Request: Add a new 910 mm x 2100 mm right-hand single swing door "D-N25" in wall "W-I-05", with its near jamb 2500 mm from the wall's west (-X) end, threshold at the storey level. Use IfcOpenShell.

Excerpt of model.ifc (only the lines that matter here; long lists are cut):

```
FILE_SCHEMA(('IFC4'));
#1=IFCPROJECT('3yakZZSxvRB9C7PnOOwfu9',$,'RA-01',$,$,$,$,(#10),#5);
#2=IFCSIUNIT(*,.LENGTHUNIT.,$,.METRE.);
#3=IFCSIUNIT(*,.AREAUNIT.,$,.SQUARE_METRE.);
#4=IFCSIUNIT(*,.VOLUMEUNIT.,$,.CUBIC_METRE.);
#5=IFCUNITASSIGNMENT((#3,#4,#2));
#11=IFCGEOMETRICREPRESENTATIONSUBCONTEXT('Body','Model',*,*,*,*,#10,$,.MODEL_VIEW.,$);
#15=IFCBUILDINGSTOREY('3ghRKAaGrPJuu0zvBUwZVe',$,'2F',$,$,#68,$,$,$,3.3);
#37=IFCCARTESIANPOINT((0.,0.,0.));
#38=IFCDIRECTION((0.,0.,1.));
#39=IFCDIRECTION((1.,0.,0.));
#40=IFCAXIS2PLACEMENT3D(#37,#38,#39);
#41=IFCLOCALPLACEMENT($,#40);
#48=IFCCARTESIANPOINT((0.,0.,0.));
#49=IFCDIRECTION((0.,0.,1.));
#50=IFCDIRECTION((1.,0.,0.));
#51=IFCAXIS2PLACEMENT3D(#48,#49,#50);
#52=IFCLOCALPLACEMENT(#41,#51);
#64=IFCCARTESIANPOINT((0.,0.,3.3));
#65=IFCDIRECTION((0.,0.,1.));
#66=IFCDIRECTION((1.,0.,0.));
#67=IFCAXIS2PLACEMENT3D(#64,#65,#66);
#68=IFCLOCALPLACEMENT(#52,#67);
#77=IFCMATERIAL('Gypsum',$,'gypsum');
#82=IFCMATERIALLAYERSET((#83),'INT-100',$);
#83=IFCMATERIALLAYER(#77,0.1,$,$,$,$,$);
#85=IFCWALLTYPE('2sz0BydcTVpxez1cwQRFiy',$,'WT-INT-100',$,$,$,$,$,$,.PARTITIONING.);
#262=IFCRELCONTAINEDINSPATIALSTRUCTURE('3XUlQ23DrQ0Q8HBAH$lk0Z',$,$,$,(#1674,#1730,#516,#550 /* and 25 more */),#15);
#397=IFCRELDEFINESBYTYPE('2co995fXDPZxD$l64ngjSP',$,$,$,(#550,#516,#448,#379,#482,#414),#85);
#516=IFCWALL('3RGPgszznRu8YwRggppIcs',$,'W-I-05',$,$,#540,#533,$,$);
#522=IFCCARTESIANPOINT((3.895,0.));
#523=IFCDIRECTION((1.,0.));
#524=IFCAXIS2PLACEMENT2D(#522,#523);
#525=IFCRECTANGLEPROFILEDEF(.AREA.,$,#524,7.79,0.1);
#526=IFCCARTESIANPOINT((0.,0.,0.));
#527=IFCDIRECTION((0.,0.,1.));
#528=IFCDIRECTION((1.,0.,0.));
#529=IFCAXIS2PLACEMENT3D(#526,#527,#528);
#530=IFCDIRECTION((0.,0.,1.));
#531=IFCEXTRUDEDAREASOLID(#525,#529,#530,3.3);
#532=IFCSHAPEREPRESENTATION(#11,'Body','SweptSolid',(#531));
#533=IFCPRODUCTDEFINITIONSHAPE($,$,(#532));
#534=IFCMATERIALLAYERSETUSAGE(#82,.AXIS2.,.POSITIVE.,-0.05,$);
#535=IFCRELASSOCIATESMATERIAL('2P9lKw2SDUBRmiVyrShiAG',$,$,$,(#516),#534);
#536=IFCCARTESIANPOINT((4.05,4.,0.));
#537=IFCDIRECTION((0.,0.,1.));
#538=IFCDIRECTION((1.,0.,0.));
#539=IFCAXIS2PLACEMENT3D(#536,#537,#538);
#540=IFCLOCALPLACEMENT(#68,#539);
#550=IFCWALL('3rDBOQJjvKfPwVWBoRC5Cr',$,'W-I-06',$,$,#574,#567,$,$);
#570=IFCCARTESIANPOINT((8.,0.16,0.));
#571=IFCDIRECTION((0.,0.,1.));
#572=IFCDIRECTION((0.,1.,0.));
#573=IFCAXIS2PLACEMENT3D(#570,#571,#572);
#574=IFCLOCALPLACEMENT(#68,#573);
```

```python
import numpy as np
import ifcopenshell
import ifcopenshell.api.feature
import ifcopenshell.api.geometry
import ifcopenshell.api.root
import ifcopenshell.api.spatial
import ifcopenshell.geom
import ifcopenshell.util.element
import ifcopenshell.util.placement
import ifcopenshell.util.representation
import ifcopenshell.util.shape
import ifcopenshell.util.unit

model = ifcopenshell.open("model.ifc")
unit_scale = ifcopenshell.util.unit.calculate_unit_scale(model)
settings = ifcopenshell.geom.settings()


def volume(element):
    """Net volume in cubic metres, openings subtracted."""
    shape = ifcopenshell.geom.create_shape(settings, element)
    return ifcopenshell.util.shape.get_volume(shape.geometry)


wall = model.by_guid("3RGPgszznRu8YwRggppIcs")
storey = ifcopenshell.util.element.get_container(wall, ifc_class="IfcBuildingStorey")
context = ifcopenshell.util.representation.get_context(model, "Model", "Body", "MODEL_VIEW")
before = volume(wall)

width, height, from_end, sill = 0.91, 2.1, 2.5, 0.0  # metres

# The wall runs along its own X axis, and the end named is its -X end.
wall_shape = ifcopenshell.geom.create_shape(settings, wall)
x, y, z = ifcopenshell.util.shape.get_vertices(wall_shape.geometry).T
start = x.min() + from_end
face, thickness = float(y.min()), float(y.max() - y.min())
wall_matrix = ifcopenshell.util.placement.get_local_placement(wall.ObjectPlacement)
level = ifcopenshell.util.placement.get_local_placement(storey.ObjectPlacement)[2, 3]


def in_wall(x, y):
    """Placement at x, y metres in the wall's axes, at sill height."""
    matrix = wall_matrix.copy()
    matrix[:, 3] = wall_matrix @ np.array([x / unit_scale, y / unit_scale, 0.0, 1.0])
    matrix[2, 3] = level + sill / unit_scale
    return matrix


# Opening: a box that overshoots both wall faces by 50 mm.
opening = ifcopenshell.api.root.create_entity(model, ifc_class="IfcOpeningElement", predefined_type="OPENING")
box = ifcopenshell.api.geometry.add_wall_representation(
    model, context=context, length=width, height=height, thickness=thickness + 0.1
)
ifcopenshell.api.geometry.assign_representation(model, product=opening, representation=box)
ifcopenshell.api.geometry.edit_object_placement(model, product=opening, matrix=in_wall(start, face - 0.05), is_si=False)
ifcopenshell.api.feature.add_feature(model, feature=opening, element=wall)

door = ifcopenshell.api.root.create_entity(model, ifc_class="IfcDoor", name="D-N25", predefined_type="DOOR")
door.OverallWidth, door.OverallHeight = width / unit_scale, height / unit_scale
door.OperationType = "SINGLE_SWING_RIGHT"
body = ifcopenshell.api.geometry.add_door_representation(
    model,
    context=context,
    overall_width=door.OverallWidth,
    overall_height=door.OverallHeight,
    operation_type="SINGLE_SWING_RIGHT",
    lining_properties={"LiningDepth": thickness / unit_scale, "ThresholdDepth": thickness / unit_scale},
)
ifcopenshell.api.geometry.assign_representation(model, product=door, representation=body)
ifcopenshell.api.spatial.assign_container(model, products=[door], relating_structure=storey)
ifcopenshell.api.feature.add_filling(model, opening=opening, element=door)

# The lining spans the wall, so the door starts at the wall face.
ifcopenshell.api.geometry.edit_object_placement(model, product=door, matrix=in_wall(start, face), is_si=False)

after = volume(wall)

print(f"wall volume {before:.3f} -> {after:.3f} m3")

model.write("model_updated.ifc")
```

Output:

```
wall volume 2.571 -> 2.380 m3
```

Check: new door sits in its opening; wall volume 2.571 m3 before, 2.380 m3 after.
